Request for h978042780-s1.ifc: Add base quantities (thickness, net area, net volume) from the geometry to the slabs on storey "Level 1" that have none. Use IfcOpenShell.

First a look at what the model holds.

```python
import ifcopenshell
import ifcopenshell.util.element
import ifcopenshell.util.unit

model = ifcopenshell.open("h978042780-s1.ifc")
print(model.schema)
for unit_type in ("LENGTHUNIT", "AREAUNIT", "VOLUMEUNIT"):
    print(unit_type, ifcopenshell.util.unit.calculate_unit_scale(model, unit_type))
storey = next(s for s in model.by_type("IfcBuildingStorey") if s.Name == "Level 1")
slabs = [e for e in ifcopenshell.util.element.get_decomposition(storey) if e.is_a("IfcSlab")]
for e in sorted(slabs, key=lambda e: e.id()):
    print(e.id(), e.is_a(), e.Name, list(ifcopenshell.util.element.get_psets(e, qtos_only=True)), sep=" | ")
```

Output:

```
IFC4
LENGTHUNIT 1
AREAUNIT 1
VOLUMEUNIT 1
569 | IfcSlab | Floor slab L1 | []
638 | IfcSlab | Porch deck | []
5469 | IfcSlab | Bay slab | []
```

```python
import ifcopenshell
import ifcopenshell.api.pset
import ifcopenshell.geom
import ifcopenshell.util.element
import ifcopenshell.util.shape
import ifcopenshell.util.unit

model = ifcopenshell.open("h978042780-s1.ifc")
unit_scale = ifcopenshell.util.unit.calculate_unit_scale(model)
area_scale = ifcopenshell.util.unit.calculate_unit_scale(model, "AREAUNIT")
volume_scale = ifcopenshell.util.unit.calculate_unit_scale(model, "VOLUMEUNIT")
settings = ifcopenshell.geom.settings()

storey = next(s for s in model.by_type("IfcBuildingStorey") if s.Name == "Level 1")
slabs = [e for e in ifcopenshell.util.element.get_decomposition(storey) if e.is_a("IfcSlab")]

for e in sorted(slabs, key=lambda e: e.id()):
    if ifcopenshell.util.element.get_psets(e, qtos_only=True, should_inherit=False):
        continue
    # Geometry comes back in metres, in the element's own axes.
    shape = ifcopenshell.geom.create_shape(settings, e)
    values = {
        "Width": ifcopenshell.util.shape.get_z(shape.geometry) / unit_scale,
        "NetArea": ifcopenshell.util.shape.get_footprint_area(shape.geometry) / area_scale,
        "NetVolume": ifcopenshell.util.shape.get_volume(shape.geometry) / volume_scale,
    }
    qto = ifcopenshell.api.pset.add_qto(model, product=e, name="Qto_SlabBaseQuantities")
    ifcopenshell.api.pset.edit_qto(model, qto=qto, properties=values)
    print(e.id(), {k: round(v, 3) for k, v in values.items()})

model.write("h978042780-s1-out.ifc")
```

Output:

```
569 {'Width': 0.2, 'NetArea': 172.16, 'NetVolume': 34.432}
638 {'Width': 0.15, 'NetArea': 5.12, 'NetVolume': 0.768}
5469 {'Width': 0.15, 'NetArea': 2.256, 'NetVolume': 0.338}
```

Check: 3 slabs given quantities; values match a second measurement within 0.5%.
